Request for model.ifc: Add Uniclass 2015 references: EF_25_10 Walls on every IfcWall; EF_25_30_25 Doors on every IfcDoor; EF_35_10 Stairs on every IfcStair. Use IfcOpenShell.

First a look at what the model holds.

```python
import ifcopenshell

model = ifcopenshell.open("model.ifc")
print(model.schema)
print("classifications:", [c.Name for c in model.by_type("IfcClassification")])
for ifc_class in ("IfcDoor", "IfcRoof", "IfcStair", "IfcWall", "IfcWindow"):
    print(ifc_class, len(model.by_type(ifc_class)))
```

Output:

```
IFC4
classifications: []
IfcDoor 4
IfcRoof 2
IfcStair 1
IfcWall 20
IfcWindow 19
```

```python
import ifcopenshell
import ifcopenshell.api.classification

model = ifcopenshell.open("model.ifc")

system = ifcopenshell.api.classification.add_classification(model, classification="Uniclass 2015")

codes = {
    "IfcWall": ("EF_25_10", "Walls"),
    "IfcDoor": ("EF_25_30_25", "Doors"),
    "IfcStair": ("EF_35_10", "Stairs"),
}
for ifc_class, (code, name) in codes.items():
    products = model.by_type(ifc_class)
    ifcopenshell.api.classification.add_reference(
        model, products=products, classification=system, identification=code, name=name
    )
    print(code, len(products))

model.write("model_rev.ifc")
```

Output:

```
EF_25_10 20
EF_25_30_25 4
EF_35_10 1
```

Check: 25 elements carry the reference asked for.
